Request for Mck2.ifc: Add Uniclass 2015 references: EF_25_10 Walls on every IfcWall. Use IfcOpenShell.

First a look at what the model holds.

```python
import ifcopenshell

model = ifcopenshell.open("Mck2.ifc")
print(model.schema)
print("classifications:", [c.Name for c in model.by_type("IfcClassification")])
for ifc_class in ("IfcDoor", "IfcRoof", "IfcStair", "IfcWall", "IfcWindow"):
    print(ifc_class, len(model.by_type(ifc_class)))
```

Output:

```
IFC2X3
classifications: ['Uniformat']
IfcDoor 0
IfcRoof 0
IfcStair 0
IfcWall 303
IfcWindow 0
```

```python
import ifcopenshell
import ifcopenshell.api.classification

model = ifcopenshell.open("Mck2.ifc")

# IFC2X3 requires Source and Edition and has no link from the project to the system.
system = model.create_entity("IfcClassification", Source="NBS", Edition="2015", Name="Uniclass 2015")

codes = {
    "IfcWall": ("EF_25_10", "Walls"),
}
for ifc_class, (code, name) in codes.items():
    products = model.by_type(ifc_class)
    ifcopenshell.api.classification.add_reference(
        model, products=products, classification=system, identification=code, name=name
    )
    print(code, len(products))

model.write("Mck2-out.ifc")
```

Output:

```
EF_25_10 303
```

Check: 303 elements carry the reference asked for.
